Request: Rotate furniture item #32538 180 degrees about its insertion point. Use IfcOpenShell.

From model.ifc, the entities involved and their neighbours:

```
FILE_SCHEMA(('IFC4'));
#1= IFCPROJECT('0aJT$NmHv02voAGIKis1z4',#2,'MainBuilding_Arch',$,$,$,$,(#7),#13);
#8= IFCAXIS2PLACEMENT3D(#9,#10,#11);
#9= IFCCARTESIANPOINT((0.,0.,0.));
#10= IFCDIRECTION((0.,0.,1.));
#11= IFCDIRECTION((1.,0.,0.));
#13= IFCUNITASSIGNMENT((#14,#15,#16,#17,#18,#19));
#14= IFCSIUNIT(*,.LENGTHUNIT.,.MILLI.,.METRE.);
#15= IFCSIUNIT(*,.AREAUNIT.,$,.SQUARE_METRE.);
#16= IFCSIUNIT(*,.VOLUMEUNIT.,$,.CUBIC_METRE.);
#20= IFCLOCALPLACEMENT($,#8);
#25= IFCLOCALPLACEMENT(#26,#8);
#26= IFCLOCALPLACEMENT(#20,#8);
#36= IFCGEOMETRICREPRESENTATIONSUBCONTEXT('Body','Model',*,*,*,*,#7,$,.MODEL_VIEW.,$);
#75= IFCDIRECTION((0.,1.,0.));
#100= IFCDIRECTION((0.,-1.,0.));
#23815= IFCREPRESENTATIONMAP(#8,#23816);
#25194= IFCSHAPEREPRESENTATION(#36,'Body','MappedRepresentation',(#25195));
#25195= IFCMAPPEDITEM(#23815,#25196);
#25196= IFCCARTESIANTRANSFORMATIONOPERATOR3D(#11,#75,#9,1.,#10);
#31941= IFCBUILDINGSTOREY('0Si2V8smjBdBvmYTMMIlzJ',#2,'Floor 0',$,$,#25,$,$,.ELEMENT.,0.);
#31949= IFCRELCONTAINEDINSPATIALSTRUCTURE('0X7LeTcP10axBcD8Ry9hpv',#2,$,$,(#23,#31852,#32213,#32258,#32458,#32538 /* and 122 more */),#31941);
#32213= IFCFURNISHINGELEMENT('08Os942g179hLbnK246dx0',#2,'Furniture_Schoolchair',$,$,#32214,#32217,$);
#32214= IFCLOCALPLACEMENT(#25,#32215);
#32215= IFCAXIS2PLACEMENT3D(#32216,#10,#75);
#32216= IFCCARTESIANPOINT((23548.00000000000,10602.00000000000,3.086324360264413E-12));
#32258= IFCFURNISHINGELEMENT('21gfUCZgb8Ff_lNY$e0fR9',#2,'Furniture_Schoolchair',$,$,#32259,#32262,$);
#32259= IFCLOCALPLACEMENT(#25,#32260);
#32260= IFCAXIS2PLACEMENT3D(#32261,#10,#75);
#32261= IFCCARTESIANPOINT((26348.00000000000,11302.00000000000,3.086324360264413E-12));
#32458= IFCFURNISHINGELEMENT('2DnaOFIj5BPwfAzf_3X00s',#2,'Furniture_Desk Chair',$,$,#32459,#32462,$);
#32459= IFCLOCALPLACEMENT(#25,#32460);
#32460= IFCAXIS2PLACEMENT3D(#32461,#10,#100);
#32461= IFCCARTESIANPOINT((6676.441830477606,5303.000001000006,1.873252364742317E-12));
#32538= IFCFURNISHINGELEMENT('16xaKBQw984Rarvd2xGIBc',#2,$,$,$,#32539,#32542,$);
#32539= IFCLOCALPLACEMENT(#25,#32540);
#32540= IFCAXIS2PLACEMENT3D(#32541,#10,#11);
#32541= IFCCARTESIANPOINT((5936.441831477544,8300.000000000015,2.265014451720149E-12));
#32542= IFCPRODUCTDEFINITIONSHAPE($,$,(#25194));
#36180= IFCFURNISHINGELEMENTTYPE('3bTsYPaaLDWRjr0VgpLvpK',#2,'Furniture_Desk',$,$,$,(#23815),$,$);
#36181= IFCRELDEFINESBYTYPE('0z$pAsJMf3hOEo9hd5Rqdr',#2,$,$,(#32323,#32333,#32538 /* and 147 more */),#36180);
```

```python
import ifcopenshell
import ifcopenshell.api.geometry
import ifcopenshell.util.placement

model = ifcopenshell.open("model.ifc")

item = model.by_guid("16xaKBQw984Rarvd2xGIBc")
matrix = ifcopenshell.util.placement.get_local_placement(item.ObjectPlacement)
matrix = matrix @ ifcopenshell.util.placement.rotation(180, "Z")
ifcopenshell.api.geometry.edit_object_placement(model, product=item, matrix=matrix, is_si=False)

print(ifcopenshell.util.placement.get_local_placement(item.ObjectPlacement).round(3) + 0.0)

model.write("model_edited.ifc")
```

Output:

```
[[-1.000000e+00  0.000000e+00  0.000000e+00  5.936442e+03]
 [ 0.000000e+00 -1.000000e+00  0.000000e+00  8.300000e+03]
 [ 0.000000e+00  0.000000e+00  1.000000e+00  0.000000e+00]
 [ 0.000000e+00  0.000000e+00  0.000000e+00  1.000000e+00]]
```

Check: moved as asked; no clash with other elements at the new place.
